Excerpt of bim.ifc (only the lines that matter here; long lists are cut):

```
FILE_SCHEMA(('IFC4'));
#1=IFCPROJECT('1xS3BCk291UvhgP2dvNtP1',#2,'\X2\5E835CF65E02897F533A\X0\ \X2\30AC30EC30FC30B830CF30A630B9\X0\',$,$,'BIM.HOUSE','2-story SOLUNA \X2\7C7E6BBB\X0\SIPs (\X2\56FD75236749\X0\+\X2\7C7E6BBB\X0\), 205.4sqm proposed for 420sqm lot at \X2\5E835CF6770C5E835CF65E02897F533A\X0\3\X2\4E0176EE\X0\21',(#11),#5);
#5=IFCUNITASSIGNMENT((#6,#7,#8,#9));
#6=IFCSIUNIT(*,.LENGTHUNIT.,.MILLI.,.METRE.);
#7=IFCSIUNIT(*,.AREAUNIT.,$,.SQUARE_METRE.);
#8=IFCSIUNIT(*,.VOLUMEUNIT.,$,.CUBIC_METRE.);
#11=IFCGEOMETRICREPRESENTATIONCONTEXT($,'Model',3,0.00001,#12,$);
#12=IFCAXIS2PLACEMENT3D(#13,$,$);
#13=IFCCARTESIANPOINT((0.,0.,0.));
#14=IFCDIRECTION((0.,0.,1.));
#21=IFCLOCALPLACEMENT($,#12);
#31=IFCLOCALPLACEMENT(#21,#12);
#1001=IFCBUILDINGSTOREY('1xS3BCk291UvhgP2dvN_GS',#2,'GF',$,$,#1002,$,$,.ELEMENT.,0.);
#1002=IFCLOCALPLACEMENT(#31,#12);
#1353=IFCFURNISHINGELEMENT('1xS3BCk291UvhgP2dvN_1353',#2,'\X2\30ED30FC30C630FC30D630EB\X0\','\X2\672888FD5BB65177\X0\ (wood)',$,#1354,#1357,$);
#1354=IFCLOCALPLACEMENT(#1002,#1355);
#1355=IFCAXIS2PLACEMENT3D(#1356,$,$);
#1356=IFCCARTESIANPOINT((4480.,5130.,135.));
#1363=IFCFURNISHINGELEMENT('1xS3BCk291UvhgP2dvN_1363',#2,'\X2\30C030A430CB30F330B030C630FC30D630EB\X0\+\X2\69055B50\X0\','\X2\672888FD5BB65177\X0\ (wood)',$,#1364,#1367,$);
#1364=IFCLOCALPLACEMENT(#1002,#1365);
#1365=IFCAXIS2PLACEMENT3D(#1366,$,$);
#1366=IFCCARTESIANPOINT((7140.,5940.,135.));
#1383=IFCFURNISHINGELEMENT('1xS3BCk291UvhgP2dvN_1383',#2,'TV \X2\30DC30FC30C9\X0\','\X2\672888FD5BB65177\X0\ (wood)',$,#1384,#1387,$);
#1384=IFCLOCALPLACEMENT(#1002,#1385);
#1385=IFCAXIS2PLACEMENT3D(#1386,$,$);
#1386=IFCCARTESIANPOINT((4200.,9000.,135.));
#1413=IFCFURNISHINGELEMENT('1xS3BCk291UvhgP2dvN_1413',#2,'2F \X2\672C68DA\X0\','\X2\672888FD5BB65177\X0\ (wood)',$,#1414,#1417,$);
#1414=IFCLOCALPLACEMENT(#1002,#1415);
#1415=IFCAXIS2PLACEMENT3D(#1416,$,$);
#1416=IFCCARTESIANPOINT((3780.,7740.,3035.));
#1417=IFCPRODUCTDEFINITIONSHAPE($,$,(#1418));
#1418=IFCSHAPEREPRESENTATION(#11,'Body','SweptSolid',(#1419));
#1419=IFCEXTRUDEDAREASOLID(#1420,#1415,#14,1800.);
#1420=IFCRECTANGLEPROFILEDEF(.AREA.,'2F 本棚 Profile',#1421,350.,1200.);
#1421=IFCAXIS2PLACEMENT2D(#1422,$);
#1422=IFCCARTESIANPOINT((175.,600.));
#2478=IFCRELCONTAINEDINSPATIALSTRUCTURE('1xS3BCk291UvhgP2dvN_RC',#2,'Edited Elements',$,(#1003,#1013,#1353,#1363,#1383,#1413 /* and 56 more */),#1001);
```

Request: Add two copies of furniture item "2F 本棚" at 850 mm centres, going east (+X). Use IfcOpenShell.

```python
import numpy as np
import ifcopenshell
import ifcopenshell.api.geometry
import ifcopenshell.api.root
import ifcopenshell.util.element
import ifcopenshell.util.placement

model = ifcopenshell.open("bim.ifc")


def reuse_history(source, copy):
    """copy_class also copies each property set's owner history, people and application; keep the originals."""
    for rel in copy.IsDefinedBy:
        if rel.is_a("IfcRelDefinesByProperties") and (history := rel.RelatingPropertyDefinition.OwnerHistory):
            rel.RelatingPropertyDefinition.OwnerHistory = source.OwnerHistory
            ifcopenshell.util.element.remove_deep2(model, history)


source = model.by_guid("1xS3BCk291UvhgP2dvN_1413")
base = ifcopenshell.util.placement.get_local_placement(source.ObjectPlacement)
step = np.array([1.0, 0.0, 0.0]) * 850.0

for i in range(1, 3):
    copy = ifcopenshell.api.root.copy_class(model, product=source)
    copy.Representation = ifcopenshell.util.element.copy_deep(
        model, source.Representation, exclude=["IfcGeometricRepresentationContext", "IfcRepresentationMap"]
    )
    reuse_history(source, copy)
    matrix = base.copy()
    matrix[:3, 3] += i * step
    print("added at", matrix[:3, 3].round(3) + 0.0)
    ifcopenshell.api.geometry.edit_object_placement(model, product=copy, matrix=matrix, is_si=False)

model.write("bim_edited.ifc")
```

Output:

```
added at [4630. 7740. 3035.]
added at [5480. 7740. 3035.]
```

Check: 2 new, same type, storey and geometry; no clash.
